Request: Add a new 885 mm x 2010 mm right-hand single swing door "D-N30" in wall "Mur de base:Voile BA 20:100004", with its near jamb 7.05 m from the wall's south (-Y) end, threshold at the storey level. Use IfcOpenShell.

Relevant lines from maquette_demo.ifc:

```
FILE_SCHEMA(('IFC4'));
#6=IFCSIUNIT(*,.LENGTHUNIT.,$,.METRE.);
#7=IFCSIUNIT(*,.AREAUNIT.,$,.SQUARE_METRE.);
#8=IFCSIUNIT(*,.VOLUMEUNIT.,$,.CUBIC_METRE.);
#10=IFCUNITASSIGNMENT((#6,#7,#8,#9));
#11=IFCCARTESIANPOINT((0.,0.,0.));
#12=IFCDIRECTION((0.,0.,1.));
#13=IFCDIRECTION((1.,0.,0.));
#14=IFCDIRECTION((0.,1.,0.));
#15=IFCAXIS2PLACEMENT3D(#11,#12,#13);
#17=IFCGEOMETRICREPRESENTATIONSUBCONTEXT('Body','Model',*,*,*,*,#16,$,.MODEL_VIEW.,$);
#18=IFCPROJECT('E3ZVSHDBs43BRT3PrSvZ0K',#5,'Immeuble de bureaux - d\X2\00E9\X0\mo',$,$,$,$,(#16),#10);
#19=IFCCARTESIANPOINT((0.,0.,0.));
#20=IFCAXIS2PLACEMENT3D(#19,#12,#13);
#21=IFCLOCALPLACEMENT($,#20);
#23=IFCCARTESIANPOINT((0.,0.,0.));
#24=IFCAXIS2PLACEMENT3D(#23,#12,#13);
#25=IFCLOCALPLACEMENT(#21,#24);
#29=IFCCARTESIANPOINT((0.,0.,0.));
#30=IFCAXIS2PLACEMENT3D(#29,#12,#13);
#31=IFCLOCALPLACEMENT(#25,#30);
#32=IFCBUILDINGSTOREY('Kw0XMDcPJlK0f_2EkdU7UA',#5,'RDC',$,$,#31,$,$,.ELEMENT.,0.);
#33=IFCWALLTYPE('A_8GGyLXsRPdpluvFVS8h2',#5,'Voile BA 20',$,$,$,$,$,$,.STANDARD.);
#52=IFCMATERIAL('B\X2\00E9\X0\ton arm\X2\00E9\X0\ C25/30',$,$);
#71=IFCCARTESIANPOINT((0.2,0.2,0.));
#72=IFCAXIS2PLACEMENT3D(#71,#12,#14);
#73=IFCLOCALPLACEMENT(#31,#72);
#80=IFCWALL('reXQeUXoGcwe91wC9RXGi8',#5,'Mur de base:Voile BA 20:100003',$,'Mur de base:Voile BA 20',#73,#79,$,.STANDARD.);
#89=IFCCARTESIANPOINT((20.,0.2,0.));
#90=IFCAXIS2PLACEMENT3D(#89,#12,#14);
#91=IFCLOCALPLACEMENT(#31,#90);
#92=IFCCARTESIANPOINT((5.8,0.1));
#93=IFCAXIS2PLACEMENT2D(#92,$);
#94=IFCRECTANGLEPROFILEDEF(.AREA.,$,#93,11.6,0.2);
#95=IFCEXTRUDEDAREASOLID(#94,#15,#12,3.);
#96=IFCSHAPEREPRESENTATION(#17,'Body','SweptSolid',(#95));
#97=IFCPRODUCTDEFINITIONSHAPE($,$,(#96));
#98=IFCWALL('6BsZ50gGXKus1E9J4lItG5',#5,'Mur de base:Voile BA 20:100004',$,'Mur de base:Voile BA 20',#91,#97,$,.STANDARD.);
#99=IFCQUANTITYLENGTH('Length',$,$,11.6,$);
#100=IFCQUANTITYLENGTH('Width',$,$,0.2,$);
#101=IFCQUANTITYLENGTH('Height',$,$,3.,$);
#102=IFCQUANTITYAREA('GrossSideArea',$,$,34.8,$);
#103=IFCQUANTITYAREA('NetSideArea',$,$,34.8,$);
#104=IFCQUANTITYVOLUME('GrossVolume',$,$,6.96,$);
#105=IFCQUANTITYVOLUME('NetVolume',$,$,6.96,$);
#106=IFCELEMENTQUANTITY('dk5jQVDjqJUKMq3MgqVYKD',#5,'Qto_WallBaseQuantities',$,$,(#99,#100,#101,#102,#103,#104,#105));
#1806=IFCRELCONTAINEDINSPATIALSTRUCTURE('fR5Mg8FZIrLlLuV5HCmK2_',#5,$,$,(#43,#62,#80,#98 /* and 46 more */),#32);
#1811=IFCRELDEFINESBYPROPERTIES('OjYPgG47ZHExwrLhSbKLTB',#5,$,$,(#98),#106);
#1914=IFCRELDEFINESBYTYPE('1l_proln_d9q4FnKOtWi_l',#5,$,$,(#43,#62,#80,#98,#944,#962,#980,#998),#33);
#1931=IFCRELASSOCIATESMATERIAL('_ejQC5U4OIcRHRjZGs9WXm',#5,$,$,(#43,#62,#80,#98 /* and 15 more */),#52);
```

```python
import numpy as np
import ifcopenshell
import ifcopenshell.api.feature
import ifcopenshell.api.geometry
import ifcopenshell.api.pset
import ifcopenshell.api.root
import ifcopenshell.api.spatial
import ifcopenshell.geom
import ifcopenshell.util.element
import ifcopenshell.util.placement
import ifcopenshell.util.representation
import ifcopenshell.util.shape
import ifcopenshell.util.unit

model = ifcopenshell.open("maquette_demo.ifc")
unit_scale = ifcopenshell.util.unit.calculate_unit_scale(model)
area_scale = ifcopenshell.util.unit.calculate_unit_scale(model, "AREAUNIT")
volume_scale = ifcopenshell.util.unit.calculate_unit_scale(model, "VOLUMEUNIT")
settings = ifcopenshell.geom.settings()


def volume(element):
    """Net volume in cubic metres, openings subtracted."""
    shape = ifcopenshell.geom.create_shape(settings, element)
    return ifcopenshell.util.shape.get_volume(shape.geometry)


wall = model.by_id(98)
storey = ifcopenshell.util.element.get_container(wall, ifc_class="IfcBuildingStorey")
context = ifcopenshell.util.representation.get_context(model, "Model", "Body", "MODEL_VIEW")
before = volume(wall)

width, height, from_end, sill = 0.885, 2.01, 7.05, 0.0  # metres

# The wall runs along its own X axis, and the end named is its -X end.
wall_shape = ifcopenshell.geom.create_shape(settings, wall)
x, y, z = ifcopenshell.util.shape.get_vertices(wall_shape.geometry).T
start = x.min() + from_end
face, thickness = float(y.min()), float(y.max() - y.min())
wall_matrix = ifcopenshell.util.placement.get_local_placement(wall.ObjectPlacement)
level = ifcopenshell.util.placement.get_local_placement(storey.ObjectPlacement)[2, 3]


def in_wall(x, y):
    """Placement at x, y metres in the wall's axes, at sill height."""
    matrix = wall_matrix.copy()
    matrix[:, 3] = wall_matrix @ np.array([x / unit_scale, y / unit_scale, 0.0, 1.0])
    matrix[2, 3] = level + sill / unit_scale
    return matrix


# Opening: a box that overshoots both wall faces by 50 mm.
opening = ifcopenshell.api.root.create_entity(model, ifc_class="IfcOpeningElement", predefined_type="OPENING")
box = ifcopenshell.api.geometry.add_wall_representation(
    model, context=context, length=width, height=height, thickness=thickness + 0.1
)
ifcopenshell.api.geometry.assign_representation(model, product=opening, representation=box)
ifcopenshell.api.geometry.edit_object_placement(model, product=opening, matrix=in_wall(start, face - 0.05), is_si=False)
ifcopenshell.api.feature.add_feature(model, feature=opening, element=wall)

door = ifcopenshell.api.root.create_entity(model, ifc_class="IfcDoor", name="D-N30", predefined_type="DOOR")
door.OverallWidth, door.OverallHeight = width / unit_scale, height / unit_scale
door.OperationType = "SINGLE_SWING_RIGHT"
body = ifcopenshell.api.geometry.add_door_representation(
    model,
    context=context,
    overall_width=door.OverallWidth,
    overall_height=door.OverallHeight,
    operation_type="SINGLE_SWING_RIGHT",
    lining_properties={"LiningDepth": thickness / unit_scale, "ThresholdDepth": thickness / unit_scale},
)
ifcopenshell.api.geometry.assign_representation(model, product=door, representation=body)
ifcopenshell.api.spatial.assign_container(model, products=[door], relating_structure=storey)
ifcopenshell.api.feature.add_filling(model, opening=opening, element=door)

# The lining spans the wall, so the door starts at the wall face.
ifcopenshell.api.geometry.edit_object_placement(model, product=door, matrix=in_wall(start, face), is_si=False)

after = volume(wall)

# Update the wall's stored quantities.
qto = model.by_id(ifcopenshell.util.element.get_pset(wall, "Qto_WallBaseQuantities", should_inherit=False)["id"])
ifcopenshell.api.pset.edit_qto(model, qto=qto, properties={
    "NetSideArea": after / thickness / area_scale,
    "NetVolume": after / volume_scale,
})

print(f"wall volume {before:.3f} -> {after:.3f} m3")

model.write("maquette_demo-out.ifc")
```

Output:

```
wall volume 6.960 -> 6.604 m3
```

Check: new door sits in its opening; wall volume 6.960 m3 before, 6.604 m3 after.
